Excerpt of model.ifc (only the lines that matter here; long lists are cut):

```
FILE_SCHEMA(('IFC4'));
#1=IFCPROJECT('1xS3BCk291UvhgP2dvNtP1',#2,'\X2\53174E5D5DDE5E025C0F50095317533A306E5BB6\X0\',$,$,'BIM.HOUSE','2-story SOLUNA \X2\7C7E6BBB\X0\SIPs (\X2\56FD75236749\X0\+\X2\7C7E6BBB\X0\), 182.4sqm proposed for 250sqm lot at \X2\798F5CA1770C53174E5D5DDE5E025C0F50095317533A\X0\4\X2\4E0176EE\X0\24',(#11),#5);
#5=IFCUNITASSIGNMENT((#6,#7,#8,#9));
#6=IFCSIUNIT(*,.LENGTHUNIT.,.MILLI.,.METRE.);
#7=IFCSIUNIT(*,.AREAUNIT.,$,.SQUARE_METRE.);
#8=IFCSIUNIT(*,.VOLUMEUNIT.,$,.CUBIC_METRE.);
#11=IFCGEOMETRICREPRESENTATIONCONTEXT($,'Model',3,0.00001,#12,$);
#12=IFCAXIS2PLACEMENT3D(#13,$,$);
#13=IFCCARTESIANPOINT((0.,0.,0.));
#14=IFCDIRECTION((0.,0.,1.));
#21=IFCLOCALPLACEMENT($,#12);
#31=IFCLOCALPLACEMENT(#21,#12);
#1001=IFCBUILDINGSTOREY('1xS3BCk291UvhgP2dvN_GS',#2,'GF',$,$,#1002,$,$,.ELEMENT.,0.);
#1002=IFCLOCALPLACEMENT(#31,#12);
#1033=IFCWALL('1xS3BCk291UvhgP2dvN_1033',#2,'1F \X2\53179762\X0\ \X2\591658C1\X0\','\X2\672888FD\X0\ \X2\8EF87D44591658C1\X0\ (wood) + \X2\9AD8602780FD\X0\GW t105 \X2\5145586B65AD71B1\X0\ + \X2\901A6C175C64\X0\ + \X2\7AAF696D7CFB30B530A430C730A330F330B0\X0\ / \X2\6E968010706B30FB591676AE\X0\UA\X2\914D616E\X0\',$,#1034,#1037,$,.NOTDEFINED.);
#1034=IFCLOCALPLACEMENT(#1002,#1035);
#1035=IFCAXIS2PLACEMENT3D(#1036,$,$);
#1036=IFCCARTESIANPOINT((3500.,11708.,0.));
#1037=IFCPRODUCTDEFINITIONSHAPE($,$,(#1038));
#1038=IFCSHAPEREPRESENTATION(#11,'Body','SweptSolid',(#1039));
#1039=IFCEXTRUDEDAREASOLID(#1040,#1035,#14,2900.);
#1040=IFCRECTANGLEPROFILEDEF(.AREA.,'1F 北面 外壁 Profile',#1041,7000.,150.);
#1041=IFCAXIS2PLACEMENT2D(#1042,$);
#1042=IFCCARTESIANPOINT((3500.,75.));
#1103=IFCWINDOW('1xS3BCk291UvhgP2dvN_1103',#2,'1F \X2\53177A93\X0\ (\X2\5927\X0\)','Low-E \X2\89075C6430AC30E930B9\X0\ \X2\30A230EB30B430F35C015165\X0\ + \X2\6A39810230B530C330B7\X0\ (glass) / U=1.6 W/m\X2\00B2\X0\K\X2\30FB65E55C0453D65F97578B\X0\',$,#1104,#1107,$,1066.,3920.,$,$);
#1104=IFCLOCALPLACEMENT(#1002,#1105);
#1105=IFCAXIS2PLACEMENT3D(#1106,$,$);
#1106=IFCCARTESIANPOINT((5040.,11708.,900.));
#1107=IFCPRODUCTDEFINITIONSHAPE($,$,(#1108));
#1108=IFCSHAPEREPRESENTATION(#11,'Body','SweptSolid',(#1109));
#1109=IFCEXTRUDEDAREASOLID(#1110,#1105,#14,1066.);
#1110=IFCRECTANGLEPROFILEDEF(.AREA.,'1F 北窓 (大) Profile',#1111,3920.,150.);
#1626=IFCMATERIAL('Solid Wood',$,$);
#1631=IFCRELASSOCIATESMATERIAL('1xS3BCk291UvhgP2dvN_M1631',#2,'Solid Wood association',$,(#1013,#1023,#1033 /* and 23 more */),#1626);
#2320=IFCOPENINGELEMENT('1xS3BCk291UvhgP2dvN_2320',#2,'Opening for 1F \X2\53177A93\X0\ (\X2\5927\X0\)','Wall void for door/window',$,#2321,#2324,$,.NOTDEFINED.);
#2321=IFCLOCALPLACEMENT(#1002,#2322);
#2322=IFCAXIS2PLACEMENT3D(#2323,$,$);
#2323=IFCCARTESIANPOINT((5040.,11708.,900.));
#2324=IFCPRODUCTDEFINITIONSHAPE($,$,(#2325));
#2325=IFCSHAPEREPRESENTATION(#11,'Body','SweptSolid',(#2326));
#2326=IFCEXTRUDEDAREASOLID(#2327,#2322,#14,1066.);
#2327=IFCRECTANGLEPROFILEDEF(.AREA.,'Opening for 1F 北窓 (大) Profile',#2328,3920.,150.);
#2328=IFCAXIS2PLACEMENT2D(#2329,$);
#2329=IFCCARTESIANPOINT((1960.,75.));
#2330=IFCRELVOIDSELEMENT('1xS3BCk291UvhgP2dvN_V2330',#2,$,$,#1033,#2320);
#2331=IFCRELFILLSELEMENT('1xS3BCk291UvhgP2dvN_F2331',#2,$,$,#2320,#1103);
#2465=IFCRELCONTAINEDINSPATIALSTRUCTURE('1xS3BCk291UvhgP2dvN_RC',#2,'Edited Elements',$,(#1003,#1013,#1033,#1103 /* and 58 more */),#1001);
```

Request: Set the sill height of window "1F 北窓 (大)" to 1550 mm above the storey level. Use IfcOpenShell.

```python
import numpy as np
import ifcopenshell
import ifcopenshell.api.geometry
import ifcopenshell.geom
import ifcopenshell.util.element
import ifcopenshell.util.placement
import ifcopenshell.util.shape
import ifcopenshell.util.unit

model = ifcopenshell.open("model.ifc")
unit_scale = ifcopenshell.util.unit.calculate_unit_scale(model)

window = model.by_id(1103)
opening = window.FillsVoids[0].RelatingOpeningElement
storey = ifcopenshell.util.element.get_container(window, ifc_class="IfcBuildingStorey")
level = ifcopenshell.util.placement.get_local_placement(storey.ObjectPlacement)[2, 3]

# The opening's origin need not be at the sill, so measure its lowest point.
shape = ifcopenshell.geom.create_shape(ifcopenshell.geom.settings(), opening)
bottom = ifcopenshell.util.shape.get_shape_bottom_elevation(shape, shape.geometry) / unit_scale
dz = level + 1.55 / unit_scale - bottom

shift = np.array([0.0, 0.0, dz])
# The window is not placed relative to its opening, so move both.
for product in (opening, window):
    matrix = ifcopenshell.util.placement.get_local_placement(product.ObjectPlacement)
    matrix[:3, 3] += shift
    ifcopenshell.api.geometry.edit_object_placement(model, product=product, matrix=matrix, is_si=False)

print(f"moved by {dz * unit_scale:+.3f} m")

model.write("model-out.ifc")
```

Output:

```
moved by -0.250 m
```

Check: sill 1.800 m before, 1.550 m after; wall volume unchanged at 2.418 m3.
